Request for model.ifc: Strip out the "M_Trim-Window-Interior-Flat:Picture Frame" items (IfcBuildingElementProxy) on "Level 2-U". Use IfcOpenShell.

First a look at what the model holds.

```python
import ifcopenshell
import ifcopenshell.util.element

model = ifcopenshell.open("model.ifc")
print(model.schema)
storey = next(s for s in model.by_type("IfcBuildingStorey") if s.Name == "Level 2-U")
proxies = [e for e in ifcopenshell.util.element.get_decomposition(storey) if e.is_a("IfcBuildingElementProxy")]
seen = {}
for e in proxies:
    element_type = ifcopenshell.util.element.get_type(e)
    name = element_type.Name if element_type not in (None, e) else None
    seen[name] = seen.get(name, 0) + 1
for name, count in sorted(seen.items(), key=str):
    print(count, "x", name)
```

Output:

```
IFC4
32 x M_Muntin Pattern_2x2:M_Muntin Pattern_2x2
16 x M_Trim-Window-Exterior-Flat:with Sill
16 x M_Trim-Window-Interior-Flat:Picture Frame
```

```python
import ifcopenshell
import ifcopenshell.api.root
import ifcopenshell.util.element

model = ifcopenshell.open("model.ifc")

storey = next(s for s in model.by_type("IfcBuildingStorey") if s.Name == "Level 2-U")
proxies = [e for e in ifcopenshell.util.element.get_decomposition(storey) if e.is_a("IfcBuildingElementProxy")]
targets = [e for e in proxies if (t := ifcopenshell.util.element.get_type(e)) not in (None, e) and t.Name == "M_Trim-Window-Interior-Flat:Picture Frame"]

for e in targets:
    ifcopenshell.api.root.remove_product(model, product=e)
print(len(targets), "removed")

model.write("model_edited.ifc")
```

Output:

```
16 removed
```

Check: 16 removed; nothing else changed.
